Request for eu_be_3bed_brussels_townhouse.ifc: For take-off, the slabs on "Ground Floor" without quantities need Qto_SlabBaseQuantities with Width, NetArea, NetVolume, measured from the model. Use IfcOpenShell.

First a look at what the model holds.

```python
import ifcopenshell
import ifcopenshell.util.element
import ifcopenshell.util.unit

model = ifcopenshell.open("eu_be_3bed_brussels_townhouse.ifc")
print(model.schema)
for unit_type in ("LENGTHUNIT", "AREAUNIT", "VOLUMEUNIT"):
    print(unit_type, ifcopenshell.util.unit.calculate_unit_scale(model, unit_type))
storey = next(s for s in model.by_type("IfcBuildingStorey") if s.Name == "Ground Floor")
slabs = [e for e in ifcopenshell.util.element.get_decomposition(storey) if e.is_a("IfcSlab")]
for e in sorted(slabs, key=lambda e: e.id()):
    print(e.id(), e.is_a(), e.Name, list(ifcopenshell.util.element.get_psets(e, qtos_only=True)), sep=" | ")
```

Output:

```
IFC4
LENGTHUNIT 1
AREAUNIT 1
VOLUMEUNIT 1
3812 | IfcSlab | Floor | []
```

```python
import ifcopenshell
import ifcopenshell.api.pset
import ifcopenshell.geom
import ifcopenshell.util.element
import ifcopenshell.util.shape
import ifcopenshell.util.unit

model = ifcopenshell.open("eu_be_3bed_brussels_townhouse.ifc")
unit_scale = ifcopenshell.util.unit.calculate_unit_scale(model)
area_scale = ifcopenshell.util.unit.calculate_unit_scale(model, "AREAUNIT")
volume_scale = ifcopenshell.util.unit.calculate_unit_scale(model, "VOLUMEUNIT")
settings = ifcopenshell.geom.settings()

storey = next(s for s in model.by_type("IfcBuildingStorey") if s.Name == "Ground Floor")
slabs = [e for e in ifcopenshell.util.element.get_decomposition(storey) if e.is_a("IfcSlab")]

for e in sorted(slabs, key=lambda e: e.id()):
    if ifcopenshell.util.element.get_psets(e, qtos_only=True, should_inherit=False):
        continue
    # Geometry comes back in metres, in the element's own axes.
    shape = ifcopenshell.geom.create_shape(settings, e)
    values = {
        "Width": ifcopenshell.util.shape.get_z(shape.geometry) / unit_scale,
        "NetArea": ifcopenshell.util.shape.get_footprint_area(shape.geometry) / area_scale,
        "NetVolume": ifcopenshell.util.shape.get_volume(shape.geometry) / volume_scale,
    }
    qto = ifcopenshell.api.pset.add_qto(model, product=e, name="Qto_SlabBaseQuantities")
    ifcopenshell.api.pset.edit_qto(model, qto=qto, properties=values)
    print(e.id(), {k: round(v, 3) for k, v in values.items()})

model.write("eu_be_3bed_brussels_townhouse-out.ifc")
```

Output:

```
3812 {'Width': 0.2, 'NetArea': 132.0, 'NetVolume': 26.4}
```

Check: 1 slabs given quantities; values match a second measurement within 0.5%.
